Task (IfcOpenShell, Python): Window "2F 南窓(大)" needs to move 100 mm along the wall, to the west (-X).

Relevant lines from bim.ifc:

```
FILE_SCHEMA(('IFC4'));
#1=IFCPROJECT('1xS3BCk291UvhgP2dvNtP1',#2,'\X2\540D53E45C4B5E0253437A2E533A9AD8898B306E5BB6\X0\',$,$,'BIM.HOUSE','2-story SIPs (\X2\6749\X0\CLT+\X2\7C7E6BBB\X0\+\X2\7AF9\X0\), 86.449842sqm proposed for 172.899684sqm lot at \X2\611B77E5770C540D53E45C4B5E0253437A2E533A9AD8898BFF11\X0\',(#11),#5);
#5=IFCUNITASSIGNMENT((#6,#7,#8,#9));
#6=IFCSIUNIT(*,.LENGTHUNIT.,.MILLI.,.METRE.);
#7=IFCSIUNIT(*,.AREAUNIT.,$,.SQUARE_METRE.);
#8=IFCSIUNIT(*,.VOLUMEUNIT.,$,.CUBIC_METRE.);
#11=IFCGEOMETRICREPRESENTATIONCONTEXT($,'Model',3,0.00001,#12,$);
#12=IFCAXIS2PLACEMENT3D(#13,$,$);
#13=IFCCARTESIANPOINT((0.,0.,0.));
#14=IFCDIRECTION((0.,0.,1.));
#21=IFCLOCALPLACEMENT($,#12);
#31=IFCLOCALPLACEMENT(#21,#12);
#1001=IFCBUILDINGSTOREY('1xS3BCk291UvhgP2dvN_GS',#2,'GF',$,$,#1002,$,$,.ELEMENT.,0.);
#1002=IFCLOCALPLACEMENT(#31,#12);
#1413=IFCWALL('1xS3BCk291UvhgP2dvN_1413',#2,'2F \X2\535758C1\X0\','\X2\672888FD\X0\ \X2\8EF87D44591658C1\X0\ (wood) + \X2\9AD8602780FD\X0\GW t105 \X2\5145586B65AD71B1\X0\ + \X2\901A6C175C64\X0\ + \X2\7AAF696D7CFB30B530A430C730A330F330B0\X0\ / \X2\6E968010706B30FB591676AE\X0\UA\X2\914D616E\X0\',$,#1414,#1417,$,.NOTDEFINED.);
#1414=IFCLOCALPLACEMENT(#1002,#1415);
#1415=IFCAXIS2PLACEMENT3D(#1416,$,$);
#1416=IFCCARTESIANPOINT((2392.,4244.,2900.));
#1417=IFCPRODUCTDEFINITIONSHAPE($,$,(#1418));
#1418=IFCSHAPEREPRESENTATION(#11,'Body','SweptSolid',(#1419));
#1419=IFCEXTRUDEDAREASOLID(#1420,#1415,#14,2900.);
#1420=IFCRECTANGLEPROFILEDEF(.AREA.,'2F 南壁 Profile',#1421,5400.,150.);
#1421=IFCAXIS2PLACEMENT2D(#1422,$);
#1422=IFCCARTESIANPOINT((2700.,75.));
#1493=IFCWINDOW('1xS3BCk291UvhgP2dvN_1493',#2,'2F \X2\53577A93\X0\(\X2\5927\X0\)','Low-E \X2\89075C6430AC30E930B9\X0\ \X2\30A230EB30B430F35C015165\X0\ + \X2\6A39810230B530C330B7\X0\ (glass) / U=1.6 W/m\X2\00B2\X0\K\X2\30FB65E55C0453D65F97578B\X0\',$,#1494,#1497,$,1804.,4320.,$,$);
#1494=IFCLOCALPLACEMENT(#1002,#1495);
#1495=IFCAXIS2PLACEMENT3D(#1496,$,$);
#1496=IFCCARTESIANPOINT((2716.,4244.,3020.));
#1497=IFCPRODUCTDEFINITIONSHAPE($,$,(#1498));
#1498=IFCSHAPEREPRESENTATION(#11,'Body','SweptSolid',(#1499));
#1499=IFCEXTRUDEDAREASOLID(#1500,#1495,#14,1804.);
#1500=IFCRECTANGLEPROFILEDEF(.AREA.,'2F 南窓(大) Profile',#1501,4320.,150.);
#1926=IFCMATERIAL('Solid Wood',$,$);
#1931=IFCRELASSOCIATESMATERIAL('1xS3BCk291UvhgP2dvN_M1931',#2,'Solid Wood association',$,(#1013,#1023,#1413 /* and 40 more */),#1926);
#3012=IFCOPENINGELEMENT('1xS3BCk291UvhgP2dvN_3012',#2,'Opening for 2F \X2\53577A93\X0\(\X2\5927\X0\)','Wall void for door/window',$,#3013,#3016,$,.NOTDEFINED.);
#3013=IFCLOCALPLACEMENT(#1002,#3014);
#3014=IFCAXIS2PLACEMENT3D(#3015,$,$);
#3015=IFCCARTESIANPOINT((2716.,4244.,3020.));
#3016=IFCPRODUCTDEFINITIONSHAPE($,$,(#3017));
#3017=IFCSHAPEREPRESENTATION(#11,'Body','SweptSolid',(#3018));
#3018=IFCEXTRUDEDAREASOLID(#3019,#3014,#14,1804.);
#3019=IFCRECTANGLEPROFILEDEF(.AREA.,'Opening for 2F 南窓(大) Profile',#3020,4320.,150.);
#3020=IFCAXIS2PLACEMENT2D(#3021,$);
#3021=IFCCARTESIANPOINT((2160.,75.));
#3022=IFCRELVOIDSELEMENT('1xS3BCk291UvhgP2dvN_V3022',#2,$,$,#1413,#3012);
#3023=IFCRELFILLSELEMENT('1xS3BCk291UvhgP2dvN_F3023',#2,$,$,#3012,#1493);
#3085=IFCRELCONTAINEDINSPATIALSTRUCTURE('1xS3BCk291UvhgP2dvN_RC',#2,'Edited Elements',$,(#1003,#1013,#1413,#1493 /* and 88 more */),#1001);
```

```python
import ifcopenshell
import ifcopenshell.api.geometry
import ifcopenshell.util.placement

model = ifcopenshell.open("bim.ifc")

window = model.by_guid("1xS3BCk291UvhgP2dvN_1493")
opening = window.FillsVoids[0].RelatingOpeningElement
wall = opening.VoidsElements[0].RelatingBuildingElement

wall_matrix = ifcopenshell.util.placement.get_local_placement(wall.ObjectPlacement)
shift = wall_matrix[:3, 0] * -100.0
before = ifcopenshell.util.placement.get_local_placement(window.ObjectPlacement)[:3, 3].copy()

# The window is not placed relative to its opening, so move both.
for product in (opening, window):
    matrix = ifcopenshell.util.placement.get_local_placement(product.ObjectPlacement)
    matrix[:3, 3] += shift
    ifcopenshell.api.geometry.edit_object_placement(model, product=product, matrix=matrix, is_si=False)

after = ifcopenshell.util.placement.get_local_placement(window.ObjectPlacement)[:3, 3]
print("window moved by", (after - before).round(3) + 0.0)

model.write("bim-out.ifc")
```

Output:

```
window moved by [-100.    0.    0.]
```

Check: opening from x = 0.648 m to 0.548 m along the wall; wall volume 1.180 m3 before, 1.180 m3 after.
